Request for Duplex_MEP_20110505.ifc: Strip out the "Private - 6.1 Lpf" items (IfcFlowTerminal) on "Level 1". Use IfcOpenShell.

First a look at what the model holds.

```python
import ifcopenshell
import ifcopenshell.util.element

model = ifcopenshell.open("Duplex_MEP_20110505.ifc")
print(model.schema)
storey = next(s for s in model.by_type("IfcBuildingStorey") if s.Name == "Level 1")
terminals = [e for e in ifcopenshell.util.element.get_decomposition(storey) if e.is_a("IfcFlowTerminal")]
seen = {}
for e in terminals:
    element_type = ifcopenshell.util.element.get_type(e)
    name = element_type.Name if element_type not in (None, e) else None
    seen[name] = seen.get(name, 0) + 1
for name, count in sorted(seen.items(), key=str):
    print(count, "x", name)
```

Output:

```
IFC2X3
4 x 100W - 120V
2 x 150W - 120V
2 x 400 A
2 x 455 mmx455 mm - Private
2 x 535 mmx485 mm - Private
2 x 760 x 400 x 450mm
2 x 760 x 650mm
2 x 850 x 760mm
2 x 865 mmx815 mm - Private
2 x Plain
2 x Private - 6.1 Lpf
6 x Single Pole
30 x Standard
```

```python
import ifcopenshell
import ifcopenshell.api.root
import ifcopenshell.util.element

model = ifcopenshell.open("Duplex_MEP_20110505.ifc")

storey = next(s for s in model.by_type("IfcBuildingStorey") if s.Name == "Level 1")
terminals = [e for e in ifcopenshell.util.element.get_decomposition(storey) if e.is_a("IfcFlowTerminal")]
targets = [e for e in terminals if (t := ifcopenshell.util.element.get_type(e)) not in (None, e) and t.Name == "Private - 6.1 Lpf"]

for e in targets:
    ifcopenshell.api.root.remove_product(model, product=e)
print(len(targets), "removed")

model.write("Duplex_MEP_20110505_rev.ifc")
```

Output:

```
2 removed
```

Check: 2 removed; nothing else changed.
